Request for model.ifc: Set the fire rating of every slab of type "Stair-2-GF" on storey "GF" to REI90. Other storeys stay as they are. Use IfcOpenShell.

First a look at what the model holds.

```python
import ifcopenshell
import ifcopenshell.util.element

model = ifcopenshell.open("model.ifc")
print(model.schema)
storey = next(s for s in model.by_type("IfcBuildingStorey") if s.Name == "GF")
slabs = [e for e in ifcopenshell.util.element.get_decomposition(storey) if e.is_a("IfcSlab")]
seen = {}
for e in slabs:
    element_type = ifcopenshell.util.element.get_type(e)
    key = (element_type.Name if element_type != e and element_type else None, ifcopenshell.util.element.get_pset(e, "Pset_SlabCommon", "FireRating"))
    seen[key] = seen.get(key, 0) + 1
for (name, value), count in sorted(seen.items(), key=str):
    print(count, "x", name, "|", value)
```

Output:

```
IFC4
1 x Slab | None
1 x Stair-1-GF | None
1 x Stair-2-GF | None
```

```python
import ifcopenshell
import ifcopenshell.api.pset
import ifcopenshell.util.element

model = ifcopenshell.open("model.ifc")

storey = next(s for s in model.by_type("IfcBuildingStorey") if s.Name == "GF")
slabs = [e for e in ifcopenshell.util.element.get_decomposition(storey) if e.is_a("IfcSlab")]

count = 0
for e in slabs:
    element_type = ifcopenshell.util.element.get_type(e)
    if element_type in (None, e) or element_type.Name != "Stair-2-GF":
        continue
    # add_pset returns the element's existing set when there is one.
    pset = ifcopenshell.api.pset.add_pset(model, product=e, name="Pset_SlabCommon")
    ifcopenshell.api.pset.edit_pset(model, pset=pset, properties={"FireRating": "REI90"})
    count += 1

print(count, "slabs updated")

model.write("model-out.ifc")
```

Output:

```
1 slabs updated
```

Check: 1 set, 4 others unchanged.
